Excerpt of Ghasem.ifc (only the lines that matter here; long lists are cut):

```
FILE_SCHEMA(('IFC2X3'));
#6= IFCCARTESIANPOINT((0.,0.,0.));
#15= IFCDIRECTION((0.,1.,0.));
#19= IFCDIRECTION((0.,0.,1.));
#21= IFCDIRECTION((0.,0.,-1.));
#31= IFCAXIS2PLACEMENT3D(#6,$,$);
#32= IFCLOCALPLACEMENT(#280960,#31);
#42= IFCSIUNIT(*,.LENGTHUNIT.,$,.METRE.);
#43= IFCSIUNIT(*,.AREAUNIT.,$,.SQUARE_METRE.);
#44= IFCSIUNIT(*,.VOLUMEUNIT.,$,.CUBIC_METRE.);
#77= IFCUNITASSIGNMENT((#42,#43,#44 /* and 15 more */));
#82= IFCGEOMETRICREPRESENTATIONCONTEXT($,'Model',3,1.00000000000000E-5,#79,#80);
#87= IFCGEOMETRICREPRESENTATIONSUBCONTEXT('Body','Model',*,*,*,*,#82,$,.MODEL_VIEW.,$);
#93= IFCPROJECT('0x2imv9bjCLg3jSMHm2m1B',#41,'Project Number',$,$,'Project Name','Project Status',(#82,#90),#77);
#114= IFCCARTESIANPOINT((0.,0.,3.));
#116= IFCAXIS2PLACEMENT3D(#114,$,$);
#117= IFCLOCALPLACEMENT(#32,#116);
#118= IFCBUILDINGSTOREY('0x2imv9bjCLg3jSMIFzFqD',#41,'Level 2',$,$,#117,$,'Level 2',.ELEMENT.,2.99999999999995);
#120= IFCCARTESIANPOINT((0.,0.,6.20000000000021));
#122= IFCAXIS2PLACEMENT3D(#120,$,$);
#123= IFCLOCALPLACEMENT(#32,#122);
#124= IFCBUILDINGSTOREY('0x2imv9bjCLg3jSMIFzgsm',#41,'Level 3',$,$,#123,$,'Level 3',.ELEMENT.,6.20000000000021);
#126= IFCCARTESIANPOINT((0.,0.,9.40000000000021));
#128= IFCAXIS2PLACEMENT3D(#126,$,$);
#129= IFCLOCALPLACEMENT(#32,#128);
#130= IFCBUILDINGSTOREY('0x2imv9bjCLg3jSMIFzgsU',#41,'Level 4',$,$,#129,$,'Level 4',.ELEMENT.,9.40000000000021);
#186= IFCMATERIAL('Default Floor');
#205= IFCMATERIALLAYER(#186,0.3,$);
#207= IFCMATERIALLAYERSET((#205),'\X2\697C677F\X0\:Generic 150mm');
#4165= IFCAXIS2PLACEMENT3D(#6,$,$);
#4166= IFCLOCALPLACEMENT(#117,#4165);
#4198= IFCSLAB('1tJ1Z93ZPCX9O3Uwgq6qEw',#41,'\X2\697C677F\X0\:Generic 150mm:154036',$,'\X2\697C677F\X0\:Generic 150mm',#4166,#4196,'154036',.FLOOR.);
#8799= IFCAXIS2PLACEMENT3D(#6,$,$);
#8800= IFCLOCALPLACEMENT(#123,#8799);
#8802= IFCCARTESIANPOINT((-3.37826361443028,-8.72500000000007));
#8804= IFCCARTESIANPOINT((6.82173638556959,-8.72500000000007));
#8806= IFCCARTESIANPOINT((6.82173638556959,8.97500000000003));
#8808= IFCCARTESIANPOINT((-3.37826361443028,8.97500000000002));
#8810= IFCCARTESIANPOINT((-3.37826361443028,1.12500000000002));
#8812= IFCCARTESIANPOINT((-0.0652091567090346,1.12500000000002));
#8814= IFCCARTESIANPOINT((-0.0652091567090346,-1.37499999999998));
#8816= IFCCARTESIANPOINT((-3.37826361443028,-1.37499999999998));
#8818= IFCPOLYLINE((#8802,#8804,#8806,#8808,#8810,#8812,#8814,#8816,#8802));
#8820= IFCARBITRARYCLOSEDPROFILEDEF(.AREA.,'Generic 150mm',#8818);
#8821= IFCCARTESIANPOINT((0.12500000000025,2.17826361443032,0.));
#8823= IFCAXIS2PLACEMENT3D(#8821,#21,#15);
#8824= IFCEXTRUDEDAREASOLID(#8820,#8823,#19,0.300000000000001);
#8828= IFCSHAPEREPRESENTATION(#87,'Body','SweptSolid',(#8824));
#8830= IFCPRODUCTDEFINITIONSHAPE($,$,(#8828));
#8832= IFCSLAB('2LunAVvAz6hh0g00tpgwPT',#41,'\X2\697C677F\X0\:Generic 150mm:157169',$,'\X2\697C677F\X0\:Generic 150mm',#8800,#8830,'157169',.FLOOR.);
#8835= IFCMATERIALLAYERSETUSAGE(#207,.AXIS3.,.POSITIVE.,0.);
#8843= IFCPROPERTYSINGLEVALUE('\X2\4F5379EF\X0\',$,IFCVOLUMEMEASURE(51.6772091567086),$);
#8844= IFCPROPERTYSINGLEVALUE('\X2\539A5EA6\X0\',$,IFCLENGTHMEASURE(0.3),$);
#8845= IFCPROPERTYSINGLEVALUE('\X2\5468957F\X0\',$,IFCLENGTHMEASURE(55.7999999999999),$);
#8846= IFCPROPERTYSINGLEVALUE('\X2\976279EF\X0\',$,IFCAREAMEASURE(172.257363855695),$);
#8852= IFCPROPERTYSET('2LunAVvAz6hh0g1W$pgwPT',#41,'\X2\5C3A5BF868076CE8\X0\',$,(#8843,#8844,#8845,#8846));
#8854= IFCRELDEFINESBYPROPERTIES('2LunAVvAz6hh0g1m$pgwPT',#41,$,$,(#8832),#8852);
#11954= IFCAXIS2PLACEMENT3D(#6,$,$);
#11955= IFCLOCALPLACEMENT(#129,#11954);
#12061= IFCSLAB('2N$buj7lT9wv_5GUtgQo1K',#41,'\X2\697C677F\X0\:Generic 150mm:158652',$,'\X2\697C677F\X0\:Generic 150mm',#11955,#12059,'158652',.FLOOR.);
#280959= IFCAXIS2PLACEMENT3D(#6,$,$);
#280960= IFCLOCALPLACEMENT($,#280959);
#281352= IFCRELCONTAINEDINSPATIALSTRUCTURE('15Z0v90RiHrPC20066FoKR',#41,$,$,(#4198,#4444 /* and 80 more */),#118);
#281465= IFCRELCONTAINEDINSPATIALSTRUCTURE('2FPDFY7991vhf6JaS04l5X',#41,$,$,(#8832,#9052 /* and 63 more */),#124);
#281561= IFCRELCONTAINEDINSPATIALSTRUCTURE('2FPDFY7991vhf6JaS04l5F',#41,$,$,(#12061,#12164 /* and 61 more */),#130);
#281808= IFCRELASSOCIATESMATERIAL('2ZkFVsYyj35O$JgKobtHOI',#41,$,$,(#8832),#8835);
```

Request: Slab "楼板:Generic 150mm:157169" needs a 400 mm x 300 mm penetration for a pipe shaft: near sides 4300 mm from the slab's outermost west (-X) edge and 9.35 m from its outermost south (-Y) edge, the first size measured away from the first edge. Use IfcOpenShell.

```python
import numpy as np
import ifcopenshell
import ifcopenshell.api.feature
import ifcopenshell.api.geometry
import ifcopenshell.api.pset
import ifcopenshell.api.root
import ifcopenshell.geom
import ifcopenshell.util.element
import ifcopenshell.util.placement
import ifcopenshell.util.representation
import ifcopenshell.util.shape
import ifcopenshell.util.unit

model = ifcopenshell.open("Ghasem.ifc")
unit_scale = ifcopenshell.util.unit.calculate_unit_scale(model)
area_scale = ifcopenshell.util.unit.calculate_unit_scale(model, "AREAUNIT")
volume_scale = ifcopenshell.util.unit.calculate_unit_scale(model, "VOLUMEUNIT")
settings = ifcopenshell.geom.settings()


def volume(element):
    """Net volume in cubic metres, openings subtracted."""
    shape = ifcopenshell.geom.create_shape(settings, element)
    return ifcopenshell.util.shape.get_volume(shape.geometry)


slab = model.by_id(8832)
before = volume(slab)

# Extent in the slab's own axes, in metres. The edges named are its -X and -Y sides.
slab_shape = ifcopenshell.geom.create_shape(settings, slab)
vertices = ifcopenshell.util.shape.get_vertices(slab_shape.geometry)
x_min, y_min, bottom = vertices.min(axis=0)
top = vertices[:, 2].max()

opening = ifcopenshell.api.root.create_entity(model, ifc_class="IfcOpeningElement", name="Pipe shaft opening")
context = ifcopenshell.util.representation.get_context(model, "Model", "Body", "MODEL_VIEW")
width, depth = 0.4, 0.3
outline = [(0.0, 0.0), (width, 0.0), (width, depth), (0.0, depth), (0.0, 0.0)]
# Overshoot both faces by 50 mm so the cut is clean.
shape = ifcopenshell.api.geometry.add_slab_representation(
    model, context=context, depth=top - bottom + 0.1, polyline=outline
)
ifcopenshell.api.geometry.assign_representation(model, product=opening, representation=shape)

matrix = ifcopenshell.util.placement.get_local_placement(slab.ObjectPlacement)
matrix[:, 3] = matrix @ np.append(np.array([x_min + 4.3, y_min + 9.35, bottom - 0.05]) / unit_scale, 1.0)
ifcopenshell.api.geometry.edit_object_placement(model, product=opening, matrix=matrix, is_si=False)
ifcopenshell.api.feature.add_feature(model, feature=opening, element=slab)

after = volume(slab)

# Update the slab's stored quantities.
pset = model.by_id(ifcopenshell.util.element.get_pset(slab, "尺寸标注", should_inherit=False)["id"])
ifcopenshell.api.pset.edit_pset(model, pset=pset, properties={
    "体积": model.create_entity("IfcVolumeMeasure", after / volume_scale),
    "面积": model.create_entity("IfcAreaMeasure", after / (top - bottom) / area_scale),
})

print(f"slab volume {before:.3f} -> {after:.3f} m3")

model.write("Ghasem_rev.ifc")
```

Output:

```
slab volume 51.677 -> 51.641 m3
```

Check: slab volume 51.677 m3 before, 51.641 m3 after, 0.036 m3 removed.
